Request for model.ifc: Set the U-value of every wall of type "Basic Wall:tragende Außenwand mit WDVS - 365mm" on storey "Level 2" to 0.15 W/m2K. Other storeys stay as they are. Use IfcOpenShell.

First a look at what the model holds.

```python
import ifcopenshell
import ifcopenshell.util.element

model = ifcopenshell.open("model.ifc")
print(model.schema)
storey = next(s for s in model.by_type("IfcBuildingStorey") if s.Name == "Level 2")
walls = [e for e in ifcopenshell.util.element.get_decomposition(storey) if e.is_a("IfcWall")]
seen = {}
for e in walls:
    element_type = ifcopenshell.util.element.get_type(e)
    key = (element_type.Name if element_type != e and element_type else None, ifcopenshell.util.element.get_pset(e, "Pset_WallCommon", "ThermalTransmittance"))
    seen[key] = seen.get(key, 0) + 1
for (name, value), count in sorted(seen.items(), key=str):
    print(count, "x", name, "|", value)
```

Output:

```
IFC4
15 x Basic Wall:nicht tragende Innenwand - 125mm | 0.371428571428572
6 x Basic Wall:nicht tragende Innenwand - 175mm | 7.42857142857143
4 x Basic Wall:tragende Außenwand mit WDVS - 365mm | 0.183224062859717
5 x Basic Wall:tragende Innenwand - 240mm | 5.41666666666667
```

```python
import ifcopenshell
import ifcopenshell.api.pset
import ifcopenshell.util.element

model = ifcopenshell.open("model.ifc")

storey = next(s for s in model.by_type("IfcBuildingStorey") if s.Name == "Level 2")
walls = [e for e in ifcopenshell.util.element.get_decomposition(storey) if e.is_a("IfcWall")]

count = 0
for e in walls:
    element_type = ifcopenshell.util.element.get_type(e)
    if element_type in (None, e) or element_type.Name != "Basic Wall:tragende Außenwand mit WDVS - 365mm":
        continue
    # add_pset returns the element's existing set when there is one.
    pset = ifcopenshell.api.pset.add_pset(model, product=e, name="Pset_WallCommon")
    ifcopenshell.api.pset.edit_pset(model, pset=pset, properties={"ThermalTransmittance": 0.15})
    count += 1

print(count, "walls updated")

model.write("model_rev.ifc")
```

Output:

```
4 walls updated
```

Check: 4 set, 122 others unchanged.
